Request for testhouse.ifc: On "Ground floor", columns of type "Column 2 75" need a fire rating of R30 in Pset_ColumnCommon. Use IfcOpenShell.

First a look at what the model holds.

```python
import ifcopenshell
import ifcopenshell.util.element

model = ifcopenshell.open("testhouse.ifc")
print(model.schema)
storey = next(s for s in model.by_type("IfcBuildingStorey") if s.Name == "Ground floor")
columns = [e for e in ifcopenshell.util.element.get_decomposition(storey) if e.is_a("IfcColumn")]
seen = {}
for e in columns:
    element_type = ifcopenshell.util.element.get_type(e)
    key = (element_type.Name if element_type != e and element_type else None, ifcopenshell.util.element.get_pset(e, "Pset_ColumnCommon", "FireRating"))
    seen[key] = seen.get(key, 0) + 1
for (name, value), count in sorted(seen.items(), key=str):
    print(count, "x", name, "|", value)
```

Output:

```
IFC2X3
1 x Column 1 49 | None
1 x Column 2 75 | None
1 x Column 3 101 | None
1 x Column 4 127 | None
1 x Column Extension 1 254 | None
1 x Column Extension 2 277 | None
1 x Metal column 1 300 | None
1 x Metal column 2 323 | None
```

```python
import ifcopenshell
import ifcopenshell.api.pset
import ifcopenshell.util.element

model = ifcopenshell.open("testhouse.ifc")

storey = next(s for s in model.by_type("IfcBuildingStorey") if s.Name == "Ground floor")
columns = [e for e in ifcopenshell.util.element.get_decomposition(storey) if e.is_a("IfcColumn")]

count = 0
for e in columns:
    element_type = ifcopenshell.util.element.get_type(e)
    if element_type in (None, e) or element_type.Name != "Column 2 75":
        continue
    # add_pset returns the element's existing set when there is one.
    pset = ifcopenshell.api.pset.add_pset(model, product=e, name="Pset_ColumnCommon")
    ifcopenshell.api.pset.edit_pset(model, pset=pset, properties={"FireRating": "R30"})
    count += 1

print(count, "columns updated")

model.write("testhouse_v2.ifc")
```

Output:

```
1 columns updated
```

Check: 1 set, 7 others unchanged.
